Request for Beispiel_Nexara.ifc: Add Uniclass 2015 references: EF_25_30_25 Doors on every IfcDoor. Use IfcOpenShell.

First a look at what the model holds.

```python
import ifcopenshell

model = ifcopenshell.open("Beispiel_Nexara.ifc")
print(model.schema)
print("classifications:", [c.Name for c in model.by_type("IfcClassification")])
for ifc_class in ("IfcDoor", "IfcRoof", "IfcStair", "IfcWall", "IfcWindow"):
    print(ifc_class, len(model.by_type(ifc_class)))
```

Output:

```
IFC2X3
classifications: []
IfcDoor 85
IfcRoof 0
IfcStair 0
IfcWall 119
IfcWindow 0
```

```python
import ifcopenshell
import ifcopenshell.api.classification

model = ifcopenshell.open("Beispiel_Nexara.ifc")

# IFC2X3 requires Source and Edition and has no link from the project to the system.
system = model.create_entity("IfcClassification", Source="NBS", Edition="2015", Name="Uniclass 2015")

codes = {
    "IfcDoor": ("EF_25_30_25", "Doors"),
}
for ifc_class, (code, name) in codes.items():
    products = model.by_type(ifc_class)
    ifcopenshell.api.classification.add_reference(
        model, products=products, classification=system, identification=code, name=name
    )
    print(code, len(products))

model.write("Beispiel_Nexara-out.ifc")
```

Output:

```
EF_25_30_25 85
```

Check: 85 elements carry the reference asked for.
